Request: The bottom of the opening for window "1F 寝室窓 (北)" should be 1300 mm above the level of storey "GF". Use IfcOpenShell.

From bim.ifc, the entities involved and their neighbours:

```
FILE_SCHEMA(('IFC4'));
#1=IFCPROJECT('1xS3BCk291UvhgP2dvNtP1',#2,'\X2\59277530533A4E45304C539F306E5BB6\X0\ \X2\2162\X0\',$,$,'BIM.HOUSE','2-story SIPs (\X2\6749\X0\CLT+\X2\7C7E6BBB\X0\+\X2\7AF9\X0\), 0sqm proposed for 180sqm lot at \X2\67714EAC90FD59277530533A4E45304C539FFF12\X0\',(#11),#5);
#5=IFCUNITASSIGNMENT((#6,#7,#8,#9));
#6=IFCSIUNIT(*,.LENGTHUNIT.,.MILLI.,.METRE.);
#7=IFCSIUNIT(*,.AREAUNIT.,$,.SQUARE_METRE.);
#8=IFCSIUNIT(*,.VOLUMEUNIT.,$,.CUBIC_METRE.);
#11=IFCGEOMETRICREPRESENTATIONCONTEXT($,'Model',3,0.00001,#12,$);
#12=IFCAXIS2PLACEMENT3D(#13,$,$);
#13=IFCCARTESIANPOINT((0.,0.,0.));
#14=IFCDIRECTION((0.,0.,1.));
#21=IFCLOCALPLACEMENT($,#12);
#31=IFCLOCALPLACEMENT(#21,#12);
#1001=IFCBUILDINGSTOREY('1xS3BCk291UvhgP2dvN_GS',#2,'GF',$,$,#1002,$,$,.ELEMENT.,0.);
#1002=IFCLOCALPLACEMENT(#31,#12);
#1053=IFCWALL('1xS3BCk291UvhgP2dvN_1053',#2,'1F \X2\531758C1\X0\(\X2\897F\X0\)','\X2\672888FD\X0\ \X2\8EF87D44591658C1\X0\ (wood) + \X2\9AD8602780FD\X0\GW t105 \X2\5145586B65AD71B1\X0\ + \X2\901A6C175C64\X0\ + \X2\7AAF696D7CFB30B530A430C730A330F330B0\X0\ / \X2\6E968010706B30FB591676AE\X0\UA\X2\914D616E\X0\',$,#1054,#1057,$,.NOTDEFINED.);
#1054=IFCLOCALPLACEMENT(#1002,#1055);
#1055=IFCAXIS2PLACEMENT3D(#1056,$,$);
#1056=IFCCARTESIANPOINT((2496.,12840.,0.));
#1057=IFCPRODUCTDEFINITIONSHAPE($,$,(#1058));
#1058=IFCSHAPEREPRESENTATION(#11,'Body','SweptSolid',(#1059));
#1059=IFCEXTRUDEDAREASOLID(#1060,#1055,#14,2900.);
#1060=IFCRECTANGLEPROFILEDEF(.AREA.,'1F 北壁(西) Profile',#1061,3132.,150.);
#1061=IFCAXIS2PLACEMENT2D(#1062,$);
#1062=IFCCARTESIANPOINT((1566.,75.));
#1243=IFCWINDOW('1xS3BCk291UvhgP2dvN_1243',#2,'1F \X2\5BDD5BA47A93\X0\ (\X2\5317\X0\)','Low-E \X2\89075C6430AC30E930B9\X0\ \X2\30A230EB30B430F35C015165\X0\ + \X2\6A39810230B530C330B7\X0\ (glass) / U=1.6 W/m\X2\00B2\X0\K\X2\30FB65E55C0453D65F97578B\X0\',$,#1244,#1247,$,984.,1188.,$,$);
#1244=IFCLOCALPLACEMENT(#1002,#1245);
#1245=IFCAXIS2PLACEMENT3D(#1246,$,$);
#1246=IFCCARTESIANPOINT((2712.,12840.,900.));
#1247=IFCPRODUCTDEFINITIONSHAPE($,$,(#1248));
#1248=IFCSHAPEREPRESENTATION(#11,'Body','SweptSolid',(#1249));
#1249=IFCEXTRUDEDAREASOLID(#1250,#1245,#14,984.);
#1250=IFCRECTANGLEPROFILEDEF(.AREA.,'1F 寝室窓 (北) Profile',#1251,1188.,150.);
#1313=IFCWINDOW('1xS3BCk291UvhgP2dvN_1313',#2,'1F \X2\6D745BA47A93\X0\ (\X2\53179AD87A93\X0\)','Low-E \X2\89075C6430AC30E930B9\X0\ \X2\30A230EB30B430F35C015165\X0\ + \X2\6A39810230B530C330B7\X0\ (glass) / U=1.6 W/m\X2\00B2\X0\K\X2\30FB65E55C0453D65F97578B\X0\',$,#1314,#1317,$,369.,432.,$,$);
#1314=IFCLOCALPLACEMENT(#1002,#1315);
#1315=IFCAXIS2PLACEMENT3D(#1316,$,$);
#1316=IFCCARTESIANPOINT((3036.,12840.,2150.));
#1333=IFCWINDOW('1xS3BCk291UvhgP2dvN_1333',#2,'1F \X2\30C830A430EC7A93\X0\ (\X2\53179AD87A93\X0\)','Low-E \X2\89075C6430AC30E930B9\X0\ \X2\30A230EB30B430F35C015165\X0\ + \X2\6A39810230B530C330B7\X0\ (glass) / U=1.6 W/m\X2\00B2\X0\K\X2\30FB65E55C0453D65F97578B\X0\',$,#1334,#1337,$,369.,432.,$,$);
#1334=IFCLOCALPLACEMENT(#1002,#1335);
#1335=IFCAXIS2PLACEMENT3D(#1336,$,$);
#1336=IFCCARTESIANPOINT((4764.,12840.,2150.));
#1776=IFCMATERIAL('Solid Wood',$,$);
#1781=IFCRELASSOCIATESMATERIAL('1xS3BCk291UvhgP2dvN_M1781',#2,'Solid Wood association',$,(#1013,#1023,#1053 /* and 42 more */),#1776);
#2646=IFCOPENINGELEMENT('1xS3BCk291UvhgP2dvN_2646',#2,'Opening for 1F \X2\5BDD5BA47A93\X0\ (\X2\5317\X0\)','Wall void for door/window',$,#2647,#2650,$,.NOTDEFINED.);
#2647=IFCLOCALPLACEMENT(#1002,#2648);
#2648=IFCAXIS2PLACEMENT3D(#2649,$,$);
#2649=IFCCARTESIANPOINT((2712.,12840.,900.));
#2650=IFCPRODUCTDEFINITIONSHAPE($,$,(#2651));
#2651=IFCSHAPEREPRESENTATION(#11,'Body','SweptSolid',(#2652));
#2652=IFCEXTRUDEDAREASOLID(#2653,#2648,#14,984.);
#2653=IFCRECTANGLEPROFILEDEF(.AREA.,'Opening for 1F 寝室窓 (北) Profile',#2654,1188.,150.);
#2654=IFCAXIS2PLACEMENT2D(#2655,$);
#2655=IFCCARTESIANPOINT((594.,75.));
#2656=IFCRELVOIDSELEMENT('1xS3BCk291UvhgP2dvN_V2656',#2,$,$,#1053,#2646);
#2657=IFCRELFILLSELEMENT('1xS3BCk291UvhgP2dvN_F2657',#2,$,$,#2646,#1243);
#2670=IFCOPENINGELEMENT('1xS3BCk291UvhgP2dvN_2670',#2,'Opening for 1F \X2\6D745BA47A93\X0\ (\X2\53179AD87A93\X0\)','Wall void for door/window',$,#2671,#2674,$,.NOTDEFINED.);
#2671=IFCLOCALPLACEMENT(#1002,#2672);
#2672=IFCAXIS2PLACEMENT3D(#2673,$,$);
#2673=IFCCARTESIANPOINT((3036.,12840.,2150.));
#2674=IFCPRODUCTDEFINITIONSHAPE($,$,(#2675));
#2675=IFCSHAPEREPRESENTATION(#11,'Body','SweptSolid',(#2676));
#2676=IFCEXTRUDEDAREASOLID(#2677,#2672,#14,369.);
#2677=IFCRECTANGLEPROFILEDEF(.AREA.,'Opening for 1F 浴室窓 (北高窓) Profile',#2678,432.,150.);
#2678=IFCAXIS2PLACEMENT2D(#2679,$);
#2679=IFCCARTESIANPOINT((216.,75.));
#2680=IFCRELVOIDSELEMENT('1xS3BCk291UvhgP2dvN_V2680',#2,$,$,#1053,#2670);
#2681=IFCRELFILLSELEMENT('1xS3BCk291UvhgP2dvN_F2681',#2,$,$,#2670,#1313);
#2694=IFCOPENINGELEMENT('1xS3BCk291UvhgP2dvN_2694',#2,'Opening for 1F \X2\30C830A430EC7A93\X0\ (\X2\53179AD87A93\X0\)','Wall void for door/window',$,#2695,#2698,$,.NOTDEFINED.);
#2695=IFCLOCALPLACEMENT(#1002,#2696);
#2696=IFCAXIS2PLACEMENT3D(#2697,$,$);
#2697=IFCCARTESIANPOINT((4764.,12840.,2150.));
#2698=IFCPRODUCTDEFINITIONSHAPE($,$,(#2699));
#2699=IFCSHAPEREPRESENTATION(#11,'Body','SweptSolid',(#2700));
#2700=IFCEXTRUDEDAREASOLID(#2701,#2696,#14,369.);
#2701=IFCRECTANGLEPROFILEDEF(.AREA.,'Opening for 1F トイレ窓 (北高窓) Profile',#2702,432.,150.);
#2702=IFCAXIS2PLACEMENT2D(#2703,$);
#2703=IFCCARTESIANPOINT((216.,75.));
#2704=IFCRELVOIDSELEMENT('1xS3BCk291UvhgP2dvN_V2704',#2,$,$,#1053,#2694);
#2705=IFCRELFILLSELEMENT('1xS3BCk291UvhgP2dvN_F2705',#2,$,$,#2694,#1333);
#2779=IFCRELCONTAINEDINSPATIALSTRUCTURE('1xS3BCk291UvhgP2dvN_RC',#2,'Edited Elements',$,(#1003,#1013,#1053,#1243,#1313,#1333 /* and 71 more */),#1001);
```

```python
import numpy as np
import ifcopenshell
import ifcopenshell.api.geometry
import ifcopenshell.geom
import ifcopenshell.util.element
import ifcopenshell.util.placement
import ifcopenshell.util.shape
import ifcopenshell.util.unit

model = ifcopenshell.open("bim.ifc")
unit_scale = ifcopenshell.util.unit.calculate_unit_scale(model)

window = model.by_id(1243)
opening = window.FillsVoids[0].RelatingOpeningElement
storey = ifcopenshell.util.element.get_container(window, ifc_class="IfcBuildingStorey")
level = ifcopenshell.util.placement.get_local_placement(storey.ObjectPlacement)[2, 3]

# The opening's origin need not be at the sill, so measure its lowest point.
shape = ifcopenshell.geom.create_shape(ifcopenshell.geom.settings(), opening)
bottom = ifcopenshell.util.shape.get_shape_bottom_elevation(shape, shape.geometry) / unit_scale
dz = level + 1300.0 - bottom

shift = np.array([0.0, 0.0, dz])
# The window is not placed relative to its opening, so move both.
for product in (opening, window):
    matrix = ifcopenshell.util.placement.get_local_placement(product.ObjectPlacement)
    matrix[:3, 3] += shift
    ifcopenshell.api.geometry.edit_object_placement(model, product=product, matrix=matrix, is_si=False)

print(f"moved by {dz * unit_scale:+.3f} m")

model.write("bim_rev.ifc")
```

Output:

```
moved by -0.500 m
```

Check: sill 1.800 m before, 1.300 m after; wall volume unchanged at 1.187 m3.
